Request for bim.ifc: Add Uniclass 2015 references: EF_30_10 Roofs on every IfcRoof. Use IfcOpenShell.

First a look at what the model holds.

```python
import ifcopenshell

model = ifcopenshell.open("bim.ifc")
print(model.schema)
print("classifications:", [c.Name for c in model.by_type("IfcClassification")])
for ifc_class in ("IfcDoor", "IfcRoof", "IfcStair", "IfcWall", "IfcWindow"):
    print(ifc_class, len(model.by_type(ifc_class)))
```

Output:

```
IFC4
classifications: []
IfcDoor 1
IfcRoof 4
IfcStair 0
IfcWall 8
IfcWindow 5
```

```python
import ifcopenshell
import ifcopenshell.api.classification

model = ifcopenshell.open("bim.ifc")

system = ifcopenshell.api.classification.add_classification(model, classification="Uniclass 2015")

codes = {
    "IfcRoof": ("EF_30_10", "Roofs"),
}
for ifc_class, (code, name) in codes.items():
    products = model.by_type(ifc_class)
    ifcopenshell.api.classification.add_reference(
        model, products=products, classification=system, identification=code, name=name
    )
    print(code, len(products))

model.write("bim_v2.ifc")
```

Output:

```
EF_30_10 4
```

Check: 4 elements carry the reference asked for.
